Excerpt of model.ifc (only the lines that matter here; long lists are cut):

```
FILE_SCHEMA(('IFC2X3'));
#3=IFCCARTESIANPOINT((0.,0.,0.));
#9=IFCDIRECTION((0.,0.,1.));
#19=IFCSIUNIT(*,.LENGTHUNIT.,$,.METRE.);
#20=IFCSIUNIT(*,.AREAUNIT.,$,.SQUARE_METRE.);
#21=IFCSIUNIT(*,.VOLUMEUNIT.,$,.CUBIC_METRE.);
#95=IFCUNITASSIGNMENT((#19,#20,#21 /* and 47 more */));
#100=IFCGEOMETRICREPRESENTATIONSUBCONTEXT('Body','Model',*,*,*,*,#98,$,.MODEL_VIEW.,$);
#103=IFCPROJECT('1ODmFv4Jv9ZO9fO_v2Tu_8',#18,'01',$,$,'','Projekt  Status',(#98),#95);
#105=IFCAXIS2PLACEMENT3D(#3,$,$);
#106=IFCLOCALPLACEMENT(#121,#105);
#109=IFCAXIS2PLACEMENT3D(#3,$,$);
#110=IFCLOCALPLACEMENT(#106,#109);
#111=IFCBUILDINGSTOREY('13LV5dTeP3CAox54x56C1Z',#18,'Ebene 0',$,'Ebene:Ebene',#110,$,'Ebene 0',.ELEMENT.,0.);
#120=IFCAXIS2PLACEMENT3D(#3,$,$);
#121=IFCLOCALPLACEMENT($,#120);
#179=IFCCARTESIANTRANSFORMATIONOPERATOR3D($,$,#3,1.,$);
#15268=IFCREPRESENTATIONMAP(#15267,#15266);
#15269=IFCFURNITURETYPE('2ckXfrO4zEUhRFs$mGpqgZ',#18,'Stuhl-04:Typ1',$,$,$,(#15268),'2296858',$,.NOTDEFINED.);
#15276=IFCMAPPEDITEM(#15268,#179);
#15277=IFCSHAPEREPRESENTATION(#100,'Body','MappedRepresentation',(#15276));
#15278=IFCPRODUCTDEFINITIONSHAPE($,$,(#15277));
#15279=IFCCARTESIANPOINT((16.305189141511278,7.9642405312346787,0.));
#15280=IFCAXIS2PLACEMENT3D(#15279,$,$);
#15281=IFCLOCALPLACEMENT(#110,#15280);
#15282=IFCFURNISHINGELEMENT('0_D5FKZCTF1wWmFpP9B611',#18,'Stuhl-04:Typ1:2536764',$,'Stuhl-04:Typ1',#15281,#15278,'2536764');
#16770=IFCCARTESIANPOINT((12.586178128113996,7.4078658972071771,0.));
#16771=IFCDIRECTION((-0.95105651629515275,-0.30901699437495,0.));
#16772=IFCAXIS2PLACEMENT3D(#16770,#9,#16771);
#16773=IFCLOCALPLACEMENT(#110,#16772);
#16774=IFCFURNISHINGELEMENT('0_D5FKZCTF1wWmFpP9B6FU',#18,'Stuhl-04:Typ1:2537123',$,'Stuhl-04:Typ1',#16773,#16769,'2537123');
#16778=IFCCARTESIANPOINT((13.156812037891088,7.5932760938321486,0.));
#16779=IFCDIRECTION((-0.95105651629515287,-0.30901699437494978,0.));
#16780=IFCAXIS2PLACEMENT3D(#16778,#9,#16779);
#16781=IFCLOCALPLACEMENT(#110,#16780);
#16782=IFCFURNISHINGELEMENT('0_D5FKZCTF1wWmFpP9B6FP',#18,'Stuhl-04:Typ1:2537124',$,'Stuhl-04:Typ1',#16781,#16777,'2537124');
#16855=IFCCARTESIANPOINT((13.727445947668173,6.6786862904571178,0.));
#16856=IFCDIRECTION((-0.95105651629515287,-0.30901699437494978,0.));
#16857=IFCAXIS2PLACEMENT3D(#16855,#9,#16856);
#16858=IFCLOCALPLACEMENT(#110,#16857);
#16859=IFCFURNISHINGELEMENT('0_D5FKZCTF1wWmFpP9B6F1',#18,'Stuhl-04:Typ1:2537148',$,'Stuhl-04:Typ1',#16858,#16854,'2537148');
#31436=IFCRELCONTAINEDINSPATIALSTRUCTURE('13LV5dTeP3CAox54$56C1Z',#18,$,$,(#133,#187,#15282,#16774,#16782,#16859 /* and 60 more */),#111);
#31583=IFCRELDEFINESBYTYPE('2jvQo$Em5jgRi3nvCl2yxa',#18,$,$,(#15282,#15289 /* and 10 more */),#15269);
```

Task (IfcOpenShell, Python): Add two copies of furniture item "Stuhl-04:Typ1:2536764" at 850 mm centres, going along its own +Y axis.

```python
import ifcopenshell
import ifcopenshell.api.geometry
import ifcopenshell.api.root
import ifcopenshell.util.element
import ifcopenshell.util.placement
import ifcopenshell.util.unit

model = ifcopenshell.open("model.ifc")
unit_scale = ifcopenshell.util.unit.calculate_unit_scale(model)

source = model.by_guid("0_D5FKZCTF1wWmFpP9B611")
base = ifcopenshell.util.placement.get_local_placement(source.ObjectPlacement)
step = base[:3, 1] * 0.85 / unit_scale

for i in range(1, 3):
    copy = ifcopenshell.api.root.copy_class(model, product=source)
    copy.Representation = ifcopenshell.util.element.copy_deep(
        model, source.Representation, exclude=["IfcGeometricRepresentationContext", "IfcRepresentationMap"]
    )
    copy.Name = "Stuhl-04:Typ1"
    copy.Tag = None
    matrix = base.copy()
    matrix[:3, 3] += i * step
    print("added at", matrix[:3, 3].round(3) + 0.0)
    ifcopenshell.api.geometry.edit_object_placement(model, product=copy, matrix=matrix, is_si=False)

model.write("model-out.ifc")
```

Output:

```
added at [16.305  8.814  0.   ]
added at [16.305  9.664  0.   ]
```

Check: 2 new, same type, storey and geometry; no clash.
